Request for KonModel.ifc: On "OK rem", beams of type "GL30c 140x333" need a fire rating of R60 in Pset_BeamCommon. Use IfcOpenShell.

First a look at what the model holds.

```python
import ifcopenshell
import ifcopenshell.util.element

model = ifcopenshell.open("KonModel.ifc")
print(model.schema)
storey = next(s for s in model.by_type("IfcBuildingStorey") if s.Name == "OK rem")
beams = [e for e in ifcopenshell.util.element.get_decomposition(storey) if e.is_a("IfcBeam")]
seen = {}
for e in beams:
    element_type = ifcopenshell.util.element.get_type(e)
    key = (element_type.Name if element_type != e and element_type else None, ifcopenshell.util.element.get_pset(e, "Pset_BeamCommon", "FireRating"))
    seen[key] = seen.get(key, 0) + 1
for (name, value), count in sorted(seen.items(), key=str):
    print(count, "x", name, "|", value)
```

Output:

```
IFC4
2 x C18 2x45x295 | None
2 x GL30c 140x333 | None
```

```python
import ifcopenshell
import ifcopenshell.api.pset
import ifcopenshell.util.element

model = ifcopenshell.open("KonModel.ifc")

storey = next(s for s in model.by_type("IfcBuildingStorey") if s.Name == "OK rem")
beams = [e for e in ifcopenshell.util.element.get_decomposition(storey) if e.is_a("IfcBeam")]

count = 0
for e in beams:
    element_type = ifcopenshell.util.element.get_type(e)
    if element_type in (None, e) or element_type.Name != "GL30c 140x333":
        continue
    # add_pset returns the element's existing set when there is one.
    pset = ifcopenshell.api.pset.add_pset(model, product=e, name="Pset_BeamCommon")
    ifcopenshell.api.pset.edit_pset(model, pset=pset, properties={"FireRating": "R60"})
    count += 1

print(count, "beams updated")

model.write("KonModel_v2.ifc")
```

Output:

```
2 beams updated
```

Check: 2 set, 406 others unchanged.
